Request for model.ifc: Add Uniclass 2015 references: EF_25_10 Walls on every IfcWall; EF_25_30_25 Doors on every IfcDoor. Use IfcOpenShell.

First a look at what the model holds.

```python
import ifcopenshell

model = ifcopenshell.open("model.ifc")
print(model.schema)
print("classifications:", [c.Name for c in model.by_type("IfcClassification")])
for ifc_class in ("IfcDoor", "IfcRoof", "IfcStair", "IfcWall", "IfcWindow"):
    print(ifc_class, len(model.by_type(ifc_class)))
```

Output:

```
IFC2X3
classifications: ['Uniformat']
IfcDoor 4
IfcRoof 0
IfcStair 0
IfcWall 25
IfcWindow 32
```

```python
import ifcopenshell
import ifcopenshell.api.classification

model = ifcopenshell.open("model.ifc")

# IFC2X3 requires Source and Edition and has no link from the project to the system.
system = model.create_entity("IfcClassification", Source="NBS", Edition="2015", Name="Uniclass 2015")

codes = {
    "IfcWall": ("EF_25_10", "Walls"),
    "IfcDoor": ("EF_25_30_25", "Doors"),
}
for ifc_class, (code, name) in codes.items():
    products = model.by_type(ifc_class)
    ifcopenshell.api.classification.add_reference(
        model, products=products, classification=system, identification=code, name=name
    )
    print(code, len(products))

model.write("model-out.ifc")
```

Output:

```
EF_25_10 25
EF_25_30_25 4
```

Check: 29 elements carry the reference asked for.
